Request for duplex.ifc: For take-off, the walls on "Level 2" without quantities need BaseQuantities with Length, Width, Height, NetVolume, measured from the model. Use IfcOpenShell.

First a look at what the model holds.

```python
import ifcopenshell
import ifcopenshell.util.element
import ifcopenshell.util.unit

model = ifcopenshell.open("duplex.ifc")
print(model.schema)
for unit_type in ("LENGTHUNIT", "AREAUNIT", "VOLUMEUNIT"):
    print(unit_type, ifcopenshell.util.unit.calculate_unit_scale(model, unit_type))
storey = next(s for s in model.by_type("IfcBuildingStorey") if s.Name == "Level 2")
walls = [e for e in ifcopenshell.util.element.get_decomposition(storey) if e.is_a("IfcWall")]
for e in sorted(walls, key=lambda e: e.id()):
    print(e.id(), e.is_a(), e.Name, list(ifcopenshell.util.element.get_psets(e, qtos_only=True)), sep=" | ")
```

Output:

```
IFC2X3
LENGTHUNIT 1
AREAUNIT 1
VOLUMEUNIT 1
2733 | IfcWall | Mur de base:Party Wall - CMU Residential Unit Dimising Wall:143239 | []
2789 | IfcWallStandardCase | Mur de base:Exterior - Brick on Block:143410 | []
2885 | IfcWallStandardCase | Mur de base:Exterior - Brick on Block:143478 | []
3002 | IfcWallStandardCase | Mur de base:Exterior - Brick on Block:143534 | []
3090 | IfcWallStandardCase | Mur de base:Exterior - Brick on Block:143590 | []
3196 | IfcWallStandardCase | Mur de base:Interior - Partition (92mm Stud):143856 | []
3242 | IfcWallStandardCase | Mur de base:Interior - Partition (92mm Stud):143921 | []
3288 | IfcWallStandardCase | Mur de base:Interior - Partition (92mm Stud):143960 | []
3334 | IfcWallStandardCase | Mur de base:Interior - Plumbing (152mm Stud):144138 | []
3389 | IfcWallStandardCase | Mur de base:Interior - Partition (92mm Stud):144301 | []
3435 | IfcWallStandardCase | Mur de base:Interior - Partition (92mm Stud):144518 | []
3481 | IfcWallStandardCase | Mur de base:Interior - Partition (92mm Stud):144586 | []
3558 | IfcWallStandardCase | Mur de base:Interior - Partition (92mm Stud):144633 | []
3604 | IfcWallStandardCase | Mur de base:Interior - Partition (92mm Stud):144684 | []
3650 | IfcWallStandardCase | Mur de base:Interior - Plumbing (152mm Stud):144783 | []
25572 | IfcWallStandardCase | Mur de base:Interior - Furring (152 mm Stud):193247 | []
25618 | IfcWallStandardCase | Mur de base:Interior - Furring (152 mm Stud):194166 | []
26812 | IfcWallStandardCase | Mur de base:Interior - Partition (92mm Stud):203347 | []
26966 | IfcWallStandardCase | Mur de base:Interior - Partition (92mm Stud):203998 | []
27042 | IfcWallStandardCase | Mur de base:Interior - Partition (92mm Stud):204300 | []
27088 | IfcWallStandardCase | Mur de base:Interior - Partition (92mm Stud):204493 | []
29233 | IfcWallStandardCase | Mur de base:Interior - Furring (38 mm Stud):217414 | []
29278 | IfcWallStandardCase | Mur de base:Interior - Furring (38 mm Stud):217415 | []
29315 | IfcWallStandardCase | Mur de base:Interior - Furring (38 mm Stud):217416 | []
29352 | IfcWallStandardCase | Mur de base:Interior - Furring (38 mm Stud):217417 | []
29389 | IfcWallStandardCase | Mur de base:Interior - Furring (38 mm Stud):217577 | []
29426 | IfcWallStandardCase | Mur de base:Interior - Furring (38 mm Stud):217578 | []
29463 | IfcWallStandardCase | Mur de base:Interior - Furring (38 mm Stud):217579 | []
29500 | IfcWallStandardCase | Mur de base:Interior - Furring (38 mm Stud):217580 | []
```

```python
import ifcopenshell
import ifcopenshell.api.pset
import ifcopenshell.geom
import ifcopenshell.util.element
import ifcopenshell.util.shape
import ifcopenshell.util.unit

model = ifcopenshell.open("duplex.ifc")
unit_scale = ifcopenshell.util.unit.calculate_unit_scale(model)
volume_scale = ifcopenshell.util.unit.calculate_unit_scale(model, "VOLUMEUNIT")
settings = ifcopenshell.geom.settings()

storey = next(s for s in model.by_type("IfcBuildingStorey") if s.Name == "Level 2")
walls = [e for e in ifcopenshell.util.element.get_decomposition(storey) if e.is_a("IfcWall")]

for e in sorted(walls, key=lambda e: e.id()):
    if ifcopenshell.util.element.get_psets(e, qtos_only=True, should_inherit=False):
        continue
    # Geometry comes back in metres, in the element's own axes.
    shape = ifcopenshell.geom.create_shape(settings, e)
    values = {
        "Length": ifcopenshell.util.shape.get_x(shape.geometry) / unit_scale,
        "Width": ifcopenshell.util.shape.get_y(shape.geometry) / unit_scale,
        "Height": ifcopenshell.util.shape.get_z(shape.geometry) / unit_scale,
        "NetVolume": ifcopenshell.util.shape.get_volume(shape.geometry) / volume_scale,
    }
    qto = ifcopenshell.api.pset.add_qto(model, product=e, name="BaseQuantities")
    ifcopenshell.api.pset.edit_qto(model, qto=qto, properties=values)
    print(e.id(), {k: round(v, 3) for k, v in values.items()})

model.write("duplex-out.ifc")
```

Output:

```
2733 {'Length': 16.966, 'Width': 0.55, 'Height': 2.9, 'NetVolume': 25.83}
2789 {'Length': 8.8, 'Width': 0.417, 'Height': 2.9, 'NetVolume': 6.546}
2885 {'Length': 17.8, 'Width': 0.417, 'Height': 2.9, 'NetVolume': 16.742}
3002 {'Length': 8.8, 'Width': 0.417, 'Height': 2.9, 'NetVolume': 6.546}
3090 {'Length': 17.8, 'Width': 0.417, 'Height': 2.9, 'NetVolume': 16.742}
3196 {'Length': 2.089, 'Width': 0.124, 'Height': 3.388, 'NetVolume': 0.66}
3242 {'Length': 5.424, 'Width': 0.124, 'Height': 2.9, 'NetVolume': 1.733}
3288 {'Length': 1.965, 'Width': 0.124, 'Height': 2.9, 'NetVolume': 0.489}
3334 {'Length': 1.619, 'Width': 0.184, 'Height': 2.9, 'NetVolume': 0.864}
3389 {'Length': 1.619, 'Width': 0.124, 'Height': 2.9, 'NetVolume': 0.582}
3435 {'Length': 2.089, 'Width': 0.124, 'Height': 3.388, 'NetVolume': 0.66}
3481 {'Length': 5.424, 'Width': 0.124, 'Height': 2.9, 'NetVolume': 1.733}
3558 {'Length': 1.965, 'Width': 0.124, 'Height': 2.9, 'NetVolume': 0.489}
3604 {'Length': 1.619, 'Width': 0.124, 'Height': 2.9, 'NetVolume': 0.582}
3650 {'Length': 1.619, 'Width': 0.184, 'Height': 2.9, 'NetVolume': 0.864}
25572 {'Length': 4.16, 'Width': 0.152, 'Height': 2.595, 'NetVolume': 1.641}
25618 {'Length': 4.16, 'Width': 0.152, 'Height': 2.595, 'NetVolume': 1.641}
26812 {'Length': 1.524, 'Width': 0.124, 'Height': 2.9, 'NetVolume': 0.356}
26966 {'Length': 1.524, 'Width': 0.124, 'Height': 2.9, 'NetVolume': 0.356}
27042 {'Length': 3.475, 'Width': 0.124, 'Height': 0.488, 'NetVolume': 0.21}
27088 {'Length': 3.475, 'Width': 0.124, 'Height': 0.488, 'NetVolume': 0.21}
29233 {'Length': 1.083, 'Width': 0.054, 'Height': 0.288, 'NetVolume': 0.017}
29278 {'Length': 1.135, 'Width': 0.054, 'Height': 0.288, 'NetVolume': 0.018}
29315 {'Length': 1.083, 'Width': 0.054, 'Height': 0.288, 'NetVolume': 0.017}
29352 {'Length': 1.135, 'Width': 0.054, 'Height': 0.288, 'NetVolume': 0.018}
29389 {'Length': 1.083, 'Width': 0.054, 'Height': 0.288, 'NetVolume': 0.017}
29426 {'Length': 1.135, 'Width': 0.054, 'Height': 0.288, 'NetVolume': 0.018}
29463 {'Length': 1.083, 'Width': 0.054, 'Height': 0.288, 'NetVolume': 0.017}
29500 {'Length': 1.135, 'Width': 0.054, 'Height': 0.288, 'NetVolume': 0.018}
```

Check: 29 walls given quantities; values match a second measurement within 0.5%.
